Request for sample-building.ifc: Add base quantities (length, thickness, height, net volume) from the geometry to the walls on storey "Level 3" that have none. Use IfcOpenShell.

First a look at what the model holds.

```python
import ifcopenshell
import ifcopenshell.util.element
import ifcopenshell.util.unit

model = ifcopenshell.open("sample-building.ifc")
print(model.schema)
for unit_type in ("LENGTHUNIT", "AREAUNIT", "VOLUMEUNIT"):
    print(unit_type, ifcopenshell.util.unit.calculate_unit_scale(model, unit_type))
storey = next(s for s in model.by_type("IfcBuildingStorey") if s.Name == "Level 3")
walls = [e for e in ifcopenshell.util.element.get_decomposition(storey) if e.is_a("IfcWall")]
for e in sorted(walls, key=lambda e: e.id()):
    print(e.id(), e.is_a(), e.Name, list(ifcopenshell.util.element.get_psets(e, qtos_only=True)), sep=" | ")
```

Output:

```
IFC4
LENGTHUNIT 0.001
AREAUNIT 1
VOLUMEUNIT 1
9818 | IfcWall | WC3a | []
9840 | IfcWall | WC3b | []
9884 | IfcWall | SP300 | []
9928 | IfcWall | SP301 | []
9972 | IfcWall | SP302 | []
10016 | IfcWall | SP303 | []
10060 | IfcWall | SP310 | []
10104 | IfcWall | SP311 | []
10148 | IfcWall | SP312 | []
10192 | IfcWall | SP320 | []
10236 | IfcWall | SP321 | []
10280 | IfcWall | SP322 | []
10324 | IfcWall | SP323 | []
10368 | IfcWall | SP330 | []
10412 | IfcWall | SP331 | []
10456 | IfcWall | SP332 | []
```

```python
import ifcopenshell
import ifcopenshell.api.pset
import ifcopenshell.geom
import ifcopenshell.util.element
import ifcopenshell.util.shape
import ifcopenshell.util.unit

model = ifcopenshell.open("sample-building.ifc")
unit_scale = ifcopenshell.util.unit.calculate_unit_scale(model)
volume_scale = ifcopenshell.util.unit.calculate_unit_scale(model, "VOLUMEUNIT")
settings = ifcopenshell.geom.settings()

storey = next(s for s in model.by_type("IfcBuildingStorey") if s.Name == "Level 3")
walls = [e for e in ifcopenshell.util.element.get_decomposition(storey) if e.is_a("IfcWall")]

for e in sorted(walls, key=lambda e: e.id()):
    if ifcopenshell.util.element.get_psets(e, qtos_only=True, should_inherit=False):
        continue
    # Geometry comes back in metres, in the element's own axes.
    shape = ifcopenshell.geom.create_shape(settings, e)
    values = {
        "Length": ifcopenshell.util.shape.get_x(shape.geometry) / unit_scale,
        "Width": ifcopenshell.util.shape.get_y(shape.geometry) / unit_scale,
        "Height": ifcopenshell.util.shape.get_z(shape.geometry) / unit_scale,
        "NetVolume": ifcopenshell.util.shape.get_volume(shape.geometry) / volume_scale,
    }
    qto = ifcopenshell.api.pset.add_qto(model, product=e, name="Qto_WallBaseQuantities")
    ifcopenshell.api.pset.edit_qto(model, qto=qto, properties=values)
    print(e.id(), {k: round(v, 3) for k, v in values.items()})

model.write("sample-building_edited.ifc")
```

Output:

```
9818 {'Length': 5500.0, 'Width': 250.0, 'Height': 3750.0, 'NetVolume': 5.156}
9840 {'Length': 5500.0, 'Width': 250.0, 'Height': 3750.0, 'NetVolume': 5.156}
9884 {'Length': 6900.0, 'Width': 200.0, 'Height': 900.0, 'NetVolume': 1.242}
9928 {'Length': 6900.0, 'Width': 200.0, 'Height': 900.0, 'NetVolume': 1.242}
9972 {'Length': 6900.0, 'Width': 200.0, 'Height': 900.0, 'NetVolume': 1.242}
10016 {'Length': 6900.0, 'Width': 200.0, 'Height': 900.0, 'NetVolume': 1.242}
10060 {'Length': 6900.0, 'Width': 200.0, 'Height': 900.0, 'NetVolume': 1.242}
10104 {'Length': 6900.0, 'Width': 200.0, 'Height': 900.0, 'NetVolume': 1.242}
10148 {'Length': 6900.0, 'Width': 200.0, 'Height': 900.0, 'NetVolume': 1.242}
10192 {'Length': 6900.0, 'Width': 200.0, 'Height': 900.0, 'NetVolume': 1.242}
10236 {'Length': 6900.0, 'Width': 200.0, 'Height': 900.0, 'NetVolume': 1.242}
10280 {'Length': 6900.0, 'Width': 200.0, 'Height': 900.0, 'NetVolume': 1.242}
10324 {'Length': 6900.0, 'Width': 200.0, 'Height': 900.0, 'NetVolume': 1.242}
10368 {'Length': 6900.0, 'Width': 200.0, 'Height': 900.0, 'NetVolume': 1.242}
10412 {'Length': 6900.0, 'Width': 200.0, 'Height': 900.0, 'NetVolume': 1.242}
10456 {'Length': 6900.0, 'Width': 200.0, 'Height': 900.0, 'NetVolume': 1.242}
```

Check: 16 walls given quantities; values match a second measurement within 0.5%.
